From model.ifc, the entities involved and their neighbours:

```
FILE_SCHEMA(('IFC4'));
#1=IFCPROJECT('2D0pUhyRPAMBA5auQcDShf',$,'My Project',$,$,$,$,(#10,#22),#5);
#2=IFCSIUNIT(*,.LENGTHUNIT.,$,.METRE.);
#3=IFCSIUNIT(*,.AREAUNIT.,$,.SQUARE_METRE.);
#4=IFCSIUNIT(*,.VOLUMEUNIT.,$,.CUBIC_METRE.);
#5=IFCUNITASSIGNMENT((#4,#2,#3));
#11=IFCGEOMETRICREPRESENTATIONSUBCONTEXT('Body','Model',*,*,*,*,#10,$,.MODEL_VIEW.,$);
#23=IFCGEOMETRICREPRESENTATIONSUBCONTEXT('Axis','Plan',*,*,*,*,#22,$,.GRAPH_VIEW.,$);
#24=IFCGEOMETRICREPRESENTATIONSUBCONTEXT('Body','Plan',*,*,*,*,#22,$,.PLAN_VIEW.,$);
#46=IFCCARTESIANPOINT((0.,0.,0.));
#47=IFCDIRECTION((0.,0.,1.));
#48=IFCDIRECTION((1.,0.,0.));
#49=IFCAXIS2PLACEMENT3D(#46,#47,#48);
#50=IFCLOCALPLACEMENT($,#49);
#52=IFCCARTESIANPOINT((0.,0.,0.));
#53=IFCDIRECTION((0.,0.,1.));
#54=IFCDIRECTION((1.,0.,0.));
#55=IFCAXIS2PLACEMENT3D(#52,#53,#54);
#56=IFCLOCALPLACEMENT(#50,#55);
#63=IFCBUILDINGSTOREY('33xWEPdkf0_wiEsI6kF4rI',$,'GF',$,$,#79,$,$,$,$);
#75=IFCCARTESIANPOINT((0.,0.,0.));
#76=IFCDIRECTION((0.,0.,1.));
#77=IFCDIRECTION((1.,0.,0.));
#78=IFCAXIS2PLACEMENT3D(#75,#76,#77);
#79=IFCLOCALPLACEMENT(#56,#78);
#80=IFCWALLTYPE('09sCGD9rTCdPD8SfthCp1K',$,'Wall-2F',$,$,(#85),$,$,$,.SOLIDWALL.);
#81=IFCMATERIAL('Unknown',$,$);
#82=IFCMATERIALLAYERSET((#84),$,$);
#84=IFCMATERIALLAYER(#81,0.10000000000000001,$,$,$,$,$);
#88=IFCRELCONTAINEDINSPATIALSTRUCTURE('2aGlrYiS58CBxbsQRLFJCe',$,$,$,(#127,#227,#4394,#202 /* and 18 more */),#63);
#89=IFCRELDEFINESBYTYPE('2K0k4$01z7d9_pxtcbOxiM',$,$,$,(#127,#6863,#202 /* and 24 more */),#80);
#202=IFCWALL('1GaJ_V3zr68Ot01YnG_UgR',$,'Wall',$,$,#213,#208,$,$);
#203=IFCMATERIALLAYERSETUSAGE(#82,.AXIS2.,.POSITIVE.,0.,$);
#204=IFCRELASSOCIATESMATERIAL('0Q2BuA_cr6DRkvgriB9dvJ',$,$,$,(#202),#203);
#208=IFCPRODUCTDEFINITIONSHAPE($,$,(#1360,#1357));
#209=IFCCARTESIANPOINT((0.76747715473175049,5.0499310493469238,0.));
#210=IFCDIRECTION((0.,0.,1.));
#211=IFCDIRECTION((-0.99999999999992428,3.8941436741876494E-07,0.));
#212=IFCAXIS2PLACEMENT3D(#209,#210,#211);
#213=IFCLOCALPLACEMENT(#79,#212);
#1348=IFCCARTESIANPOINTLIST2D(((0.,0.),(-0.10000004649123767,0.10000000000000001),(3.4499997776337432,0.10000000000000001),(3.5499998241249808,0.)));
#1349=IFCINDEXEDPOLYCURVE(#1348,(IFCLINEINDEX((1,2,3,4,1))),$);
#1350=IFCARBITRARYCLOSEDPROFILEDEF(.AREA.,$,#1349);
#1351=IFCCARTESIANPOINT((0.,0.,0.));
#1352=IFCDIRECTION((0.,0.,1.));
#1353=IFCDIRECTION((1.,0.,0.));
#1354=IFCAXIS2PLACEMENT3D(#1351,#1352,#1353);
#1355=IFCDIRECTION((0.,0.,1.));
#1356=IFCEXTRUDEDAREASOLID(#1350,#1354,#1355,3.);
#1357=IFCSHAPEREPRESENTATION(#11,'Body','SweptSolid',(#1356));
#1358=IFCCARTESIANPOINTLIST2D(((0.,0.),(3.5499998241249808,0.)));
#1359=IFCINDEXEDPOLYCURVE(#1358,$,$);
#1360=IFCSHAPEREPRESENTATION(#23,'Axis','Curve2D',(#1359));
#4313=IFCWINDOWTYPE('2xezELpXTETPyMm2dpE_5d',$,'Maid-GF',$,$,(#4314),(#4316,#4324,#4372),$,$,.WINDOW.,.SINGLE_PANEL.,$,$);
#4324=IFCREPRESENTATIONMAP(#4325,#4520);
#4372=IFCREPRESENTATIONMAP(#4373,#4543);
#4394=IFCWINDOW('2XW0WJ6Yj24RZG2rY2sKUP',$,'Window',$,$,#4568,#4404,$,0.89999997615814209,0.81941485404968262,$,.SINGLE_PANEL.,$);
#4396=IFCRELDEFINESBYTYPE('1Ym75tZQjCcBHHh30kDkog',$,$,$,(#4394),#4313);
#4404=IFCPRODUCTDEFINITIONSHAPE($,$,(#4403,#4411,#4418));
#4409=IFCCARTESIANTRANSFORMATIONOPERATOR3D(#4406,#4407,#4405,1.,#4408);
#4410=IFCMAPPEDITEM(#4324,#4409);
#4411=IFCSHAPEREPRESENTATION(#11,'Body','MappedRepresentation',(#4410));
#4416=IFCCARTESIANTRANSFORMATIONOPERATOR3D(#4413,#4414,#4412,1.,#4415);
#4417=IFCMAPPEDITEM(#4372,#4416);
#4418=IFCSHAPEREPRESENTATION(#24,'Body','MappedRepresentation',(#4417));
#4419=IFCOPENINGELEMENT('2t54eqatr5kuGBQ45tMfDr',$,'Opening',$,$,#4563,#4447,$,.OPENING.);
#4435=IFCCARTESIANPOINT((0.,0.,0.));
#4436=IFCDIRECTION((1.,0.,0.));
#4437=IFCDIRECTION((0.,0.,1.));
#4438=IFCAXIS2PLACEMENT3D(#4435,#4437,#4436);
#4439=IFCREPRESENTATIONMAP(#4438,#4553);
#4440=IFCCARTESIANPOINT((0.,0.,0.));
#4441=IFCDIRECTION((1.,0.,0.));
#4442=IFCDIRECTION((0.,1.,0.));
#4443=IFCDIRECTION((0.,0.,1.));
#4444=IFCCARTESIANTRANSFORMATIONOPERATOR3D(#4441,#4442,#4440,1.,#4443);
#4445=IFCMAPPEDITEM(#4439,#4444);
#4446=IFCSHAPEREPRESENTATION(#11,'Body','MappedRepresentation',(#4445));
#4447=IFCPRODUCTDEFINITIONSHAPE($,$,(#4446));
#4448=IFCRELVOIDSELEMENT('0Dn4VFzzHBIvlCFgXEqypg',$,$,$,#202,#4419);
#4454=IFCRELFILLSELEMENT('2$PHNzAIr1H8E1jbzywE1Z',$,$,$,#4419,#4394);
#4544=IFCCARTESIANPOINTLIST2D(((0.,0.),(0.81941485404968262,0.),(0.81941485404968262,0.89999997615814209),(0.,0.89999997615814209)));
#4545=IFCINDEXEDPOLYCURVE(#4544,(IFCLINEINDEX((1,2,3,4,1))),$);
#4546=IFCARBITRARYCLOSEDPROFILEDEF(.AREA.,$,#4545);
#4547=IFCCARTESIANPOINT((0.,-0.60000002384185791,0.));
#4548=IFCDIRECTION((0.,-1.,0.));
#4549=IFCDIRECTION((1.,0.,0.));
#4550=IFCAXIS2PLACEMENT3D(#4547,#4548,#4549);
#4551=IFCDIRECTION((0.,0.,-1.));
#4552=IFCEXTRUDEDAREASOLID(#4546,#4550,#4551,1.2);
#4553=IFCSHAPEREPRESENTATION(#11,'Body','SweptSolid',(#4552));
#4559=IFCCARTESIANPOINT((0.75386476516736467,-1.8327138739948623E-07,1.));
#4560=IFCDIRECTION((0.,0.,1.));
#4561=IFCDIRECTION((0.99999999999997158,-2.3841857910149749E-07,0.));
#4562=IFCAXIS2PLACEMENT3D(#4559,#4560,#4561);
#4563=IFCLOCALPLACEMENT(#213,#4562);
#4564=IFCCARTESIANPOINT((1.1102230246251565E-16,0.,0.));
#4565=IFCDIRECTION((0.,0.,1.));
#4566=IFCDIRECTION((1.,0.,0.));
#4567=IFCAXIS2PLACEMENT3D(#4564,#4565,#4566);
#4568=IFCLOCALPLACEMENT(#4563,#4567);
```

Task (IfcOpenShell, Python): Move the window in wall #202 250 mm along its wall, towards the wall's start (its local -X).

```python
import ifcopenshell
import ifcopenshell.api.geometry
import ifcopenshell.util.placement
import ifcopenshell.util.unit

model = ifcopenshell.open("model.ifc")
unit_scale = ifcopenshell.util.unit.calculate_unit_scale(model)

window = model.by_id(4394)
opening = window.FillsVoids[0].RelatingOpeningElement
wall = opening.VoidsElements[0].RelatingBuildingElement

wall_matrix = ifcopenshell.util.placement.get_local_placement(wall.ObjectPlacement)
shift = wall_matrix[:3, 0] * -0.25 / unit_scale
before = ifcopenshell.util.placement.get_local_placement(window.ObjectPlacement)[:3, 3].copy()

# The window is placed relative to its opening, so it follows when the opening moves.
matrix = ifcopenshell.util.placement.get_local_placement(opening.ObjectPlacement)
matrix[:3, 3] += shift
ifcopenshell.api.geometry.edit_object_placement(
    model, product=opening, matrix=matrix, is_si=False, should_transform_children=True
)

after = ifcopenshell.util.placement.get_local_placement(window.ObjectPlacement)[:3, 3]
print("window moved by", (after - before).round(3) + 0.0)

model.write("model_rev.ifc")
```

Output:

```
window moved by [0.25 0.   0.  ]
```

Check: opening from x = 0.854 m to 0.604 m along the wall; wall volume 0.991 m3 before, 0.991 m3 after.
